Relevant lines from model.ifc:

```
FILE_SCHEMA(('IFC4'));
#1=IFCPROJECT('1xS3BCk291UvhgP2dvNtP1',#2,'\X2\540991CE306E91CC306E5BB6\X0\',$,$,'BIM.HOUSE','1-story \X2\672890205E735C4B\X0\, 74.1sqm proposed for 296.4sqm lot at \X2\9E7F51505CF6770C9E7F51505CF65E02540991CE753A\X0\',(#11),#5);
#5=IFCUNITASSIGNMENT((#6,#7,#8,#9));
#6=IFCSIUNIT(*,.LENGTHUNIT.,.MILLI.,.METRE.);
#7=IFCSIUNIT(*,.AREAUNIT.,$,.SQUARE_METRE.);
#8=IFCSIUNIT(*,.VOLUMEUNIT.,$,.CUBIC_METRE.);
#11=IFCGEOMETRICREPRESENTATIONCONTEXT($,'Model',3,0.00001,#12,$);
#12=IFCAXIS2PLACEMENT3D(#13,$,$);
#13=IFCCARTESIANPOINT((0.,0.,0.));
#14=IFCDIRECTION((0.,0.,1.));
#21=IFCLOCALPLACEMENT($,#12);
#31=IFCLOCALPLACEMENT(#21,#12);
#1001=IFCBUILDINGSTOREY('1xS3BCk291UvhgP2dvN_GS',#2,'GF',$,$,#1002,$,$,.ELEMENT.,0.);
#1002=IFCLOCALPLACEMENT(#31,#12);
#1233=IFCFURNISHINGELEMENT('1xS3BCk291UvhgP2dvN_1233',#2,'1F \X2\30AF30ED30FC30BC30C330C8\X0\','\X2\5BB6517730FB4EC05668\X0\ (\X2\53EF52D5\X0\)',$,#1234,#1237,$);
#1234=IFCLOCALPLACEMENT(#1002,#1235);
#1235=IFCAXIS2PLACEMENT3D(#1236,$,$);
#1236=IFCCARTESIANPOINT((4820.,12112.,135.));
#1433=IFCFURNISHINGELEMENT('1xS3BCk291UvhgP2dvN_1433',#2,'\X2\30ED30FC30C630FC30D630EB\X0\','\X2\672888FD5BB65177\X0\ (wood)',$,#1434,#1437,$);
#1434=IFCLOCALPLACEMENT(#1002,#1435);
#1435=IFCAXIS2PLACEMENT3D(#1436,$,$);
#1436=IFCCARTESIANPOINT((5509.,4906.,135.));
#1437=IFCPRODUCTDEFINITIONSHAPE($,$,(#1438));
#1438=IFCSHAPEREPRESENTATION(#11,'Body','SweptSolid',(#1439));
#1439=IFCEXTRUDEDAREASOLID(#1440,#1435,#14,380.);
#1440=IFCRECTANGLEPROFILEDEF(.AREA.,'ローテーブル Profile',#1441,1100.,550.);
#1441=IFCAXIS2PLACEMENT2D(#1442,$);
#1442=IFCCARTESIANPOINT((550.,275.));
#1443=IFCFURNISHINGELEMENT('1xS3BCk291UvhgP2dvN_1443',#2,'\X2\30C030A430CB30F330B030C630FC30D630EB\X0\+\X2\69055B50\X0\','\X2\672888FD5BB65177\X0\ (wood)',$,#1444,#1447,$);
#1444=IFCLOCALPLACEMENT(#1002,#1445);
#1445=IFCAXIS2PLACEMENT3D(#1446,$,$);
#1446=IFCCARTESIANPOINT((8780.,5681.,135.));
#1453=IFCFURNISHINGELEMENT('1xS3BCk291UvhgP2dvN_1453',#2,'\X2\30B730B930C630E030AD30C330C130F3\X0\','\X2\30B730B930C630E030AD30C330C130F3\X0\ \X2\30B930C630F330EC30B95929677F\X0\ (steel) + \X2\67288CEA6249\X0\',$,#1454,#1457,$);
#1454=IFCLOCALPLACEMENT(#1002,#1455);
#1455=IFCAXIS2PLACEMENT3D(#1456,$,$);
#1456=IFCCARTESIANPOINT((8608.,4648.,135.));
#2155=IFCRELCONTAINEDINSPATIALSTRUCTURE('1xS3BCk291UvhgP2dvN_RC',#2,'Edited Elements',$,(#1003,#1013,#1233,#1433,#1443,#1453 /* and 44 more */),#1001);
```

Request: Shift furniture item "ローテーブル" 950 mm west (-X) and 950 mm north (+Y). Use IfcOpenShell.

```python
import ifcopenshell
import ifcopenshell.api.geometry
import ifcopenshell.util.placement

model = ifcopenshell.open("model.ifc")

item = model.by_id(1433)
matrix = ifcopenshell.util.placement.get_local_placement(item.ObjectPlacement)
matrix[0, 3] -= 950.0
matrix[1, 3] += 950.0
ifcopenshell.api.geometry.edit_object_placement(model, product=item, matrix=matrix, is_si=False)

print(ifcopenshell.util.placement.get_local_placement(item.ObjectPlacement).round(3) + 0.0)

model.write("model-out.ifc")
```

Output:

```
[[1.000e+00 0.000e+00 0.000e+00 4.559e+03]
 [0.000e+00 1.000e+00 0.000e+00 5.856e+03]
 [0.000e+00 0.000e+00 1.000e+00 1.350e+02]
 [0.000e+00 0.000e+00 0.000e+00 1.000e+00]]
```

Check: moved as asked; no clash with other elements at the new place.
